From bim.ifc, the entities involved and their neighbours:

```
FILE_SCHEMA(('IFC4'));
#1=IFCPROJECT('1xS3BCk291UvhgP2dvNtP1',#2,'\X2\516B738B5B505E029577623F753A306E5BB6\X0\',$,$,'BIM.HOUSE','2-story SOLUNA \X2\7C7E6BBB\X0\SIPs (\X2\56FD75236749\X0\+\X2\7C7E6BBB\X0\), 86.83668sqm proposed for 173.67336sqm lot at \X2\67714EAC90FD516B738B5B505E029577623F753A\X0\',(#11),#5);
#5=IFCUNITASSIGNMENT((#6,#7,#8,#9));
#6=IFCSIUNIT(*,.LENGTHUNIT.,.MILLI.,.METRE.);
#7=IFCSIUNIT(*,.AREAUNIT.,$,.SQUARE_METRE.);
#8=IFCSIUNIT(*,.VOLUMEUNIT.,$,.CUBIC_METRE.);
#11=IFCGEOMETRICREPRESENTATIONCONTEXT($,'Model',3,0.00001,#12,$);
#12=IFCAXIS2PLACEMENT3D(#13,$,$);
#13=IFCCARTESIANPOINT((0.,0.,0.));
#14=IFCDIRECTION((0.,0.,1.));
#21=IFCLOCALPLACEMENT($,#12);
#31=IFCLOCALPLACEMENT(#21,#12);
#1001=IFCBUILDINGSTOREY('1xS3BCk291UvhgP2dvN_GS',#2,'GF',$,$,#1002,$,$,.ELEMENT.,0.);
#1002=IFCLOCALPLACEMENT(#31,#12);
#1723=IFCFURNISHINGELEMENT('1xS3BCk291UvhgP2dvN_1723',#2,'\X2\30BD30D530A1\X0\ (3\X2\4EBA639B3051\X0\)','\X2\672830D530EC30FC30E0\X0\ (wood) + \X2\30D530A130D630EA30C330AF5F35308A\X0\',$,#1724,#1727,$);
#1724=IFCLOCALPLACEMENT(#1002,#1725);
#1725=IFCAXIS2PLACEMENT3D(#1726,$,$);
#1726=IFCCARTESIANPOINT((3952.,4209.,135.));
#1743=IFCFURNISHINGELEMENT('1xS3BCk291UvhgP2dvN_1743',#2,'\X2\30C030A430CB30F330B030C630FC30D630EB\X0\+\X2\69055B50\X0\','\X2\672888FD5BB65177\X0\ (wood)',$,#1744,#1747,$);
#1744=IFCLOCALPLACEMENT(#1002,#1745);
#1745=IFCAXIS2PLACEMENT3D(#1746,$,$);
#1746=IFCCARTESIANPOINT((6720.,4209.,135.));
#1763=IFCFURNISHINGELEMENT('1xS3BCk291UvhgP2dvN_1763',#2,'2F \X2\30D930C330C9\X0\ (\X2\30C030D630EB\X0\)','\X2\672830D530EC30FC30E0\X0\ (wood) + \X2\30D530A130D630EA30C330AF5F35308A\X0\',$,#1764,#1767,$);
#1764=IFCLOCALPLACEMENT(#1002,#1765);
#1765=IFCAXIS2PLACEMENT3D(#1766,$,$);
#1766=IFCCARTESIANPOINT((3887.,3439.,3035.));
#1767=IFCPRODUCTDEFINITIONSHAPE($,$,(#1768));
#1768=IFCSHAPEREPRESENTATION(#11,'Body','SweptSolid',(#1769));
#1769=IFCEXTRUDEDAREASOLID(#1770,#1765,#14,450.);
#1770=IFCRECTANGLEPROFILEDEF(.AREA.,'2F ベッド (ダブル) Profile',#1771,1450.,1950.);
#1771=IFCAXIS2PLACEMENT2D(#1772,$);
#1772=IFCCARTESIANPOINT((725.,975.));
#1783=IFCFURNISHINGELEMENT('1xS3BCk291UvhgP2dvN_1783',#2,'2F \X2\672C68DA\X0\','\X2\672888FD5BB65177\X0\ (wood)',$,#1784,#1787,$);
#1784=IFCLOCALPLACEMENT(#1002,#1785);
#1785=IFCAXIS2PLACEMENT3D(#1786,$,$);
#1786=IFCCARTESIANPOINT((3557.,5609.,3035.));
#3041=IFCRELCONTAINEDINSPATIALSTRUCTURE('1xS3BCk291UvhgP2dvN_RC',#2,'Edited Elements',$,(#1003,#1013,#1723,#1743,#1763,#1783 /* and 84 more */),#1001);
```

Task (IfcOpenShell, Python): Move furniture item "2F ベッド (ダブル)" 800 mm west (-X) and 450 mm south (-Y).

```python
import ifcopenshell
import ifcopenshell.api.geometry
import ifcopenshell.util.placement
import ifcopenshell.util.unit

model = ifcopenshell.open("bim.ifc")
unit_scale = ifcopenshell.util.unit.calculate_unit_scale(model)

item = model.by_guid("1xS3BCk291UvhgP2dvN_1763")
matrix = ifcopenshell.util.placement.get_local_placement(item.ObjectPlacement)
matrix[0, 3] -= 0.8 / unit_scale
matrix[1, 3] -= 0.45 / unit_scale
ifcopenshell.api.geometry.edit_object_placement(model, product=item, matrix=matrix, is_si=False)

print(ifcopenshell.util.placement.get_local_placement(item.ObjectPlacement).round(3) + 0.0)

model.write("bim_edited.ifc")
```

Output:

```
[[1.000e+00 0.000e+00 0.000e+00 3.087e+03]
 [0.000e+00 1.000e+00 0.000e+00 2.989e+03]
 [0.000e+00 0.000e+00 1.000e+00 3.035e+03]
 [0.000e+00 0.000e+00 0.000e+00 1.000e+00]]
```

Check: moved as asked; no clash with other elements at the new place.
